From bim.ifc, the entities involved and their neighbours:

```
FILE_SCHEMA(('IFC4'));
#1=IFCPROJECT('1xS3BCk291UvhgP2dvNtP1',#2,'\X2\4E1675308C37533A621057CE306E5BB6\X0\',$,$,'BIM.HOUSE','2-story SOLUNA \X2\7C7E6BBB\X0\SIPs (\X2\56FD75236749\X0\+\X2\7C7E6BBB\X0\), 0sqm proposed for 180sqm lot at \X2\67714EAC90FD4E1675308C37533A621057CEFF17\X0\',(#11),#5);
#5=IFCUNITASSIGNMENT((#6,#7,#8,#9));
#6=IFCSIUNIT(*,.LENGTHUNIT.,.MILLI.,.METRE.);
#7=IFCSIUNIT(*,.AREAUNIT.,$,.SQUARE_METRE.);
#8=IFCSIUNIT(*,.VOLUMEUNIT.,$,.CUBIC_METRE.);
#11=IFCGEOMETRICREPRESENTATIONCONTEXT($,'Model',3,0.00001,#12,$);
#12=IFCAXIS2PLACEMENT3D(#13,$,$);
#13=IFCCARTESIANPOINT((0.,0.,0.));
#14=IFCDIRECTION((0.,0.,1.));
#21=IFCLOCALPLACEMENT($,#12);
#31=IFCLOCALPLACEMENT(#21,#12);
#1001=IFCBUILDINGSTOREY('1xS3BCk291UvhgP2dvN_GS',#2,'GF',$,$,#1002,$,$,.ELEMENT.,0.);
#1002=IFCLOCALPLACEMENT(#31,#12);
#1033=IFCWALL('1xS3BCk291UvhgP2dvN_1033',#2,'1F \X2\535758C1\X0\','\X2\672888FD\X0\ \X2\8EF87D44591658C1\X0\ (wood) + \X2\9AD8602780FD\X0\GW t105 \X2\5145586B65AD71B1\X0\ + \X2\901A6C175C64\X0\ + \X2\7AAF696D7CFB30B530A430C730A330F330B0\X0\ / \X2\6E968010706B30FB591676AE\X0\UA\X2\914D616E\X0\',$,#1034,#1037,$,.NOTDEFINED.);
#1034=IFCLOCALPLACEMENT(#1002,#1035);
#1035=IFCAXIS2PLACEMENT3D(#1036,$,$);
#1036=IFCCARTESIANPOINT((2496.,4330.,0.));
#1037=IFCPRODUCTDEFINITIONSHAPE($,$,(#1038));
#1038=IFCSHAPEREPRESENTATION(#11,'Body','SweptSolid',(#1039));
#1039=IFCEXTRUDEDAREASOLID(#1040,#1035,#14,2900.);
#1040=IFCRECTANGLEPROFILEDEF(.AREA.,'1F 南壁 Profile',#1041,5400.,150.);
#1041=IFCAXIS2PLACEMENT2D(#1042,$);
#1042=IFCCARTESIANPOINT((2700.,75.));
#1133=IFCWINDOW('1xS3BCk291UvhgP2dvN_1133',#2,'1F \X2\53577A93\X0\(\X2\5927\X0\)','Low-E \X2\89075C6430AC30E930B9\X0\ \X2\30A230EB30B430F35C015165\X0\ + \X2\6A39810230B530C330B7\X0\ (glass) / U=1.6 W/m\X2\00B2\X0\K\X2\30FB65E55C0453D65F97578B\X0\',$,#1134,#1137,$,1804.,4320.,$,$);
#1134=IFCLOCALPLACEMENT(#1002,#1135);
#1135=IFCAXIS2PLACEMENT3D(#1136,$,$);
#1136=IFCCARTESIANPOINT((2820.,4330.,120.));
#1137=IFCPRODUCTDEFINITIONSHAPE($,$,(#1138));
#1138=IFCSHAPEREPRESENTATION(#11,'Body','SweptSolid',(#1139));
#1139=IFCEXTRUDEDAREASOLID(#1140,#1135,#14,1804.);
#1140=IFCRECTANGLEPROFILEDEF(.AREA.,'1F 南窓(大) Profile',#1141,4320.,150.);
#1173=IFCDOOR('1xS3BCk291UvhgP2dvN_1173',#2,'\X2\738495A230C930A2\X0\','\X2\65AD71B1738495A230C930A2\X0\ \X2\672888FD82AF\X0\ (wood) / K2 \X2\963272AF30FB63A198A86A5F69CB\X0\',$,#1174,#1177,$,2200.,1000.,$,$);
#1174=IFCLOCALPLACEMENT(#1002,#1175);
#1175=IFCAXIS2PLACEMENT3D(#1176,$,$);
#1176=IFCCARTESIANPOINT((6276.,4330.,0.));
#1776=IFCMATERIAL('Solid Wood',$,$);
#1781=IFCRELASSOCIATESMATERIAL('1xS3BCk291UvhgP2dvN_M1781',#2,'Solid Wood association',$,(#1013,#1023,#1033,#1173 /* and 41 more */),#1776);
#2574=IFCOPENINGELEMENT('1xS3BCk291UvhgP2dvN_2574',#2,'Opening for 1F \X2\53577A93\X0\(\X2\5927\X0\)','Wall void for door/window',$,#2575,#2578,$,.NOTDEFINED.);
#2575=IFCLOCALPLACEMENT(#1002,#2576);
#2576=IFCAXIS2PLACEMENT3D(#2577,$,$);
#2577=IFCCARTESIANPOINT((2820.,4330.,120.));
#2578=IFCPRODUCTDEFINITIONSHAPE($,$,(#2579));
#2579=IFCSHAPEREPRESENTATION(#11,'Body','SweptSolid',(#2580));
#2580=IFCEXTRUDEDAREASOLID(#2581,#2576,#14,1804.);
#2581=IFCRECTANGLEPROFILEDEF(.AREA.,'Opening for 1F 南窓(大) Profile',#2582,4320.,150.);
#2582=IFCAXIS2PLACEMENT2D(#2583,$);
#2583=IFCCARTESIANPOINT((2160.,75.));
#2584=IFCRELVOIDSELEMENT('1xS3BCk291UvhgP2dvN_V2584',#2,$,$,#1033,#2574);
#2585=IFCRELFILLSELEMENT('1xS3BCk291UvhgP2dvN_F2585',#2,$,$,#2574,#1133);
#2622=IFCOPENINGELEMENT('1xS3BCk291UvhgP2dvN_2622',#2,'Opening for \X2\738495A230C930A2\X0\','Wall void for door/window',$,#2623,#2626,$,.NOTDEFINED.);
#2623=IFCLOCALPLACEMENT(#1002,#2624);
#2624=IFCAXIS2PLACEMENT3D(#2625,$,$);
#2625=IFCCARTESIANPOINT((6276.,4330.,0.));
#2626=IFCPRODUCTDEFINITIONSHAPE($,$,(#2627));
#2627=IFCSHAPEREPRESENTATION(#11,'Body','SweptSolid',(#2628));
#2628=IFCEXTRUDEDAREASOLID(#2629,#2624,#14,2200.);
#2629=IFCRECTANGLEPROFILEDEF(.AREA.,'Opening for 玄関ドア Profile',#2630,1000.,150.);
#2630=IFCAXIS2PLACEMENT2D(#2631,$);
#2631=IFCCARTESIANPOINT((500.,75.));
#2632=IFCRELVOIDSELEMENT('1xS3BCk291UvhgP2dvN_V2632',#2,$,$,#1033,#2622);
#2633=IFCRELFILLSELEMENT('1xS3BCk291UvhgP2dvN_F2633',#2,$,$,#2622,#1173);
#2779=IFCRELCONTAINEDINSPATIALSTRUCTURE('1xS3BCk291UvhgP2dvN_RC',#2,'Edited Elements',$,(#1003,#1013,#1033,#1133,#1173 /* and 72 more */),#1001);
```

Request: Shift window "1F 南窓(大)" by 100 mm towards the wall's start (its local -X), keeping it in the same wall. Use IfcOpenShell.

```python
import ifcopenshell
import ifcopenshell.api.geometry
import ifcopenshell.util.placement

model = ifcopenshell.open("bim.ifc")

window = model.by_id(1133)
opening = window.FillsVoids[0].RelatingOpeningElement
wall = opening.VoidsElements[0].RelatingBuildingElement

wall_matrix = ifcopenshell.util.placement.get_local_placement(wall.ObjectPlacement)
shift = wall_matrix[:3, 0] * -100.0
before = ifcopenshell.util.placement.get_local_placement(window.ObjectPlacement)[:3, 3].copy()

# The window is not placed relative to its opening, so move both.
for product in (opening, window):
    matrix = ifcopenshell.util.placement.get_local_placement(product.ObjectPlacement)
    matrix[:3, 3] += shift
    ifcopenshell.api.geometry.edit_object_placement(model, product=product, matrix=matrix, is_si=False)

after = ifcopenshell.util.placement.get_local_placement(window.ObjectPlacement)[:3, 3]
print("window moved by", (after - before).round(3) + 0.0)

model.write("bim-out.ifc")
```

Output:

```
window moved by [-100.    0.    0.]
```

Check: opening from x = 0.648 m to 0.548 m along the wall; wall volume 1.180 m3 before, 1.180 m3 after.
